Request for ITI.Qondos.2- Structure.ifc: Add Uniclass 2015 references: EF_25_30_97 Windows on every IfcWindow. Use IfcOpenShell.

First a look at what the model holds.

```python
import ifcopenshell

model = ifcopenshell.open("ITI.Qondos.2- Structure.ifc")
print(model.schema)
print("classifications:", [c.Name for c in model.by_type("IfcClassification")])
for ifc_class in ("IfcDoor", "IfcRoof", "IfcStair", "IfcWall", "IfcWindow"):
    print(ifc_class, len(model.by_type(ifc_class)))
```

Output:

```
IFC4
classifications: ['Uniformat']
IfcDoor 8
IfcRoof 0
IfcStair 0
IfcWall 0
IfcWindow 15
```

```python
import ifcopenshell
import ifcopenshell.api.classification

model = ifcopenshell.open("ITI.Qondos.2- Structure.ifc")

system = ifcopenshell.api.classification.add_classification(model, classification="Uniclass 2015")

codes = {
    "IfcWindow": ("EF_25_30_97", "Windows"),
}
for ifc_class, (code, name) in codes.items():
    products = model.by_type(ifc_class)
    ifcopenshell.api.classification.add_reference(
        model, products=products, classification=system, identification=code, name=name
    )
    print(code, len(products))

model.write("ITI.Qondos.2- Structure_rev.ifc")
```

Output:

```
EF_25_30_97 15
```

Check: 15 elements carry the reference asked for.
